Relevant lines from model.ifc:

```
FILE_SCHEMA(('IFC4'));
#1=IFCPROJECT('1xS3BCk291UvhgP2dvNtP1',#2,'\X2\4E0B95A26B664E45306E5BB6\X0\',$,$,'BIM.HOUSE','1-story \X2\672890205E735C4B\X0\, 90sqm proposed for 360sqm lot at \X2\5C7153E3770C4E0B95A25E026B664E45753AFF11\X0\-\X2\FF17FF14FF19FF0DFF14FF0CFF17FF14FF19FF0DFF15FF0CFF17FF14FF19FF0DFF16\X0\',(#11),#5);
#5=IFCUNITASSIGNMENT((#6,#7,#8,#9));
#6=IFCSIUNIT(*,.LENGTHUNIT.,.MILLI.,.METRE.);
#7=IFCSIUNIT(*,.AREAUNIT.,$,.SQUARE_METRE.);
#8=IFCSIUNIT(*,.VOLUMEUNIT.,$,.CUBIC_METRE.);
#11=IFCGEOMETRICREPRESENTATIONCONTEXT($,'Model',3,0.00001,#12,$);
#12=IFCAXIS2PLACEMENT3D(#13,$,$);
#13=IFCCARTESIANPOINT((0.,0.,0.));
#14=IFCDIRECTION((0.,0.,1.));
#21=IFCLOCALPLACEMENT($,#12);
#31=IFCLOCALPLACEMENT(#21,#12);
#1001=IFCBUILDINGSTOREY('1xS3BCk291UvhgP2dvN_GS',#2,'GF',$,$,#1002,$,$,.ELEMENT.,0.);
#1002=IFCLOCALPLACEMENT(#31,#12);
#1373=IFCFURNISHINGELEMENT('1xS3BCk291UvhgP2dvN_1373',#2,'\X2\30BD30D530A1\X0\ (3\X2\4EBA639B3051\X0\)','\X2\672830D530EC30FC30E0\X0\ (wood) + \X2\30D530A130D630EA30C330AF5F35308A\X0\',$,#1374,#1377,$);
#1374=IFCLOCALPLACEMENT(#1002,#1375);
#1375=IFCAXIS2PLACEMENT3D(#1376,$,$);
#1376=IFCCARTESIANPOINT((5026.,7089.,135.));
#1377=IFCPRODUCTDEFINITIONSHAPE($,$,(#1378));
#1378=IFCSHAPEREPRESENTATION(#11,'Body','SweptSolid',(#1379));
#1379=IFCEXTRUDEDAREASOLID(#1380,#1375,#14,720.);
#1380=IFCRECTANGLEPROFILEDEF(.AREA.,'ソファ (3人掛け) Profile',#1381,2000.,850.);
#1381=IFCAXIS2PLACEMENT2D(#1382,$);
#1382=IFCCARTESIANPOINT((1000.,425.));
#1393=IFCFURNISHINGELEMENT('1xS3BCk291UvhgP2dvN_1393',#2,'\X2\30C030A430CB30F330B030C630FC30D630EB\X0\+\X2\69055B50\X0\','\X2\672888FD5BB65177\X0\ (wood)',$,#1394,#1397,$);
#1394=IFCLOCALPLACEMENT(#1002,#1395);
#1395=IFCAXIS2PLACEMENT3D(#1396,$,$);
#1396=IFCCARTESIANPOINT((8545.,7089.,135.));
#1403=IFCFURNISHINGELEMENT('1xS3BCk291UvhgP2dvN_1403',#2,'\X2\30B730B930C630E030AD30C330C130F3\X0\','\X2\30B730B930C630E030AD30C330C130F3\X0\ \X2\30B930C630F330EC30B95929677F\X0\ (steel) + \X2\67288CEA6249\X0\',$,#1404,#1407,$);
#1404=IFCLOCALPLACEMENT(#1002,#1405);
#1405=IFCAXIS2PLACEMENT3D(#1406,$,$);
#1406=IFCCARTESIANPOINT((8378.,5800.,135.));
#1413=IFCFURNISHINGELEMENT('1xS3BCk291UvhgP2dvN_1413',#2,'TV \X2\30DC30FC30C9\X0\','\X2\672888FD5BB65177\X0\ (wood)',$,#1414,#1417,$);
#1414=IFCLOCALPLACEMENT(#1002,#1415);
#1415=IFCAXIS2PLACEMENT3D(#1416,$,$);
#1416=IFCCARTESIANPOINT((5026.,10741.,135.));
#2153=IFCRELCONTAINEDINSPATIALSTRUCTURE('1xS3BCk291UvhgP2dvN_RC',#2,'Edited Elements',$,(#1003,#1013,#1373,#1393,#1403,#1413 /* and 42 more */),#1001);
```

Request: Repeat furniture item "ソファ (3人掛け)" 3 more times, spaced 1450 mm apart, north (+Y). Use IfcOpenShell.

```python
import numpy as np
import ifcopenshell
import ifcopenshell.api.geometry
import ifcopenshell.api.root
import ifcopenshell.util.element
import ifcopenshell.util.placement
import ifcopenshell.util.unit

model = ifcopenshell.open("model.ifc")
unit_scale = ifcopenshell.util.unit.calculate_unit_scale(model)


def reuse_history(source, copy):
    """copy_class also copies each property set's owner history, people and application; keep the originals."""
    for rel in copy.IsDefinedBy:
        if rel.is_a("IfcRelDefinesByProperties") and (history := rel.RelatingPropertyDefinition.OwnerHistory):
            rel.RelatingPropertyDefinition.OwnerHistory = source.OwnerHistory
            ifcopenshell.util.element.remove_deep2(model, history)


source = model.by_guid("1xS3BCk291UvhgP2dvN_1373")
base = ifcopenshell.util.placement.get_local_placement(source.ObjectPlacement)
step = np.array([0.0, 1.0, 0.0]) * 1.45 / unit_scale

for i in range(1, 4):
    copy = ifcopenshell.api.root.copy_class(model, product=source)
    copy.Representation = ifcopenshell.util.element.copy_deep(
        model, source.Representation, exclude=["IfcGeometricRepresentationContext", "IfcRepresentationMap"]
    )
    reuse_history(source, copy)
    matrix = base.copy()
    matrix[:3, 3] += i * step
    print("added at", matrix[:3, 3].round(3) + 0.0)
    ifcopenshell.api.geometry.edit_object_placement(model, product=copy, matrix=matrix, is_si=False)

model.write("model_rev.ifc")
```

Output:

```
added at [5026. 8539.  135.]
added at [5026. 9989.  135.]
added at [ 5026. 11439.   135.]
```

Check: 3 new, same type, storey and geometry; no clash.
